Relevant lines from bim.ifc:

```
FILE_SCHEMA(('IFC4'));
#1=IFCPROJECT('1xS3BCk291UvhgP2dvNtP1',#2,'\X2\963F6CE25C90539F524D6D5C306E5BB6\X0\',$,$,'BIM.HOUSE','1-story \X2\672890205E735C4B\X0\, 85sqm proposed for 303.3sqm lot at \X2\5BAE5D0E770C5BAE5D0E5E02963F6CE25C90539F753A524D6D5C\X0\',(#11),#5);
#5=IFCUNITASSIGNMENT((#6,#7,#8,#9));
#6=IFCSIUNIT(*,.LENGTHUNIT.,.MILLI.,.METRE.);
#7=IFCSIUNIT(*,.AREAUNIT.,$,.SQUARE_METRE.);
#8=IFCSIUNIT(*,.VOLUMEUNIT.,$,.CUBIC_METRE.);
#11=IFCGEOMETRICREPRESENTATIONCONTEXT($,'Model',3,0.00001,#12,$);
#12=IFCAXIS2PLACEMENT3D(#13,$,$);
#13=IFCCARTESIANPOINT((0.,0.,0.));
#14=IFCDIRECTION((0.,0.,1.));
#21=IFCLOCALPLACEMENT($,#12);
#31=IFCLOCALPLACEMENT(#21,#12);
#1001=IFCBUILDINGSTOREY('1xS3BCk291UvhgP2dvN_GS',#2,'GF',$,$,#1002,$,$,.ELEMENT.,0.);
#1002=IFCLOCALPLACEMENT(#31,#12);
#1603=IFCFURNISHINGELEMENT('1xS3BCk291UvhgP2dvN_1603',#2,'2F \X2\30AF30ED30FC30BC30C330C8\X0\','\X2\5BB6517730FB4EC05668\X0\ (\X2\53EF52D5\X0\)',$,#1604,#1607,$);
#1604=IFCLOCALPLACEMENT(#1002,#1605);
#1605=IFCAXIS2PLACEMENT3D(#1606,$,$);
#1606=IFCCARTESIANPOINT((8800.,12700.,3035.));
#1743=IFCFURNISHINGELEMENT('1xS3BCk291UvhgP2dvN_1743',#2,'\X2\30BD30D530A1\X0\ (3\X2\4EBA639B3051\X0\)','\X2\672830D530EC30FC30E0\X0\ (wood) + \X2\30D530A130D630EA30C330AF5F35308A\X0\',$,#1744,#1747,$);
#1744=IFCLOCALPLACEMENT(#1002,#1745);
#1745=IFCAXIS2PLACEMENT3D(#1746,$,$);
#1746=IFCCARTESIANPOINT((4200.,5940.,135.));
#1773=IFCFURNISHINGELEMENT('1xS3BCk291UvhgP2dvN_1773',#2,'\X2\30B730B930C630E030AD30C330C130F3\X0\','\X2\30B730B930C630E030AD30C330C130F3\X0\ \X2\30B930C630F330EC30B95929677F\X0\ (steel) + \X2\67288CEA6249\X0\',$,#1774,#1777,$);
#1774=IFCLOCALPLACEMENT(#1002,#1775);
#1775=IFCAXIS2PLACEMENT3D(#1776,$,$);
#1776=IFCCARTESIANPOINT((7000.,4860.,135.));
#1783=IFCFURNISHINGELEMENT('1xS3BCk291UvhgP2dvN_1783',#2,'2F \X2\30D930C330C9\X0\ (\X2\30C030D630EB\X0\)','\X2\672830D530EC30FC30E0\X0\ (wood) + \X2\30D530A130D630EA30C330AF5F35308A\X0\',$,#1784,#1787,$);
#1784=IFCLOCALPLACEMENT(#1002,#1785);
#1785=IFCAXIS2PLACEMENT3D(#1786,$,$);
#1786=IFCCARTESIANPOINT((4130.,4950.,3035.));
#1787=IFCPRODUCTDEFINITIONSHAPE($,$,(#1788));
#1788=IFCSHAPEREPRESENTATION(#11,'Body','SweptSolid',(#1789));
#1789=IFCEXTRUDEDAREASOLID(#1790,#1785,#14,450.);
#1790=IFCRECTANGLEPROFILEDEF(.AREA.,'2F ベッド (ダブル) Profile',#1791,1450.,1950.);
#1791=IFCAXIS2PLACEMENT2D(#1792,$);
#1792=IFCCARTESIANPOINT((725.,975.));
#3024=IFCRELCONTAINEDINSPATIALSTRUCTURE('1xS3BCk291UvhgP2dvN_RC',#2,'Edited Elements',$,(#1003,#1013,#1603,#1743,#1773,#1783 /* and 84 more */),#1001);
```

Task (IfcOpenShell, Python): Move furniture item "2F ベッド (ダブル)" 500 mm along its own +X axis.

```python
import ifcopenshell
import ifcopenshell.api.geometry
import ifcopenshell.util.placement

model = ifcopenshell.open("bim.ifc")

item = model.by_guid("1xS3BCk291UvhgP2dvN_1783")
matrix = ifcopenshell.util.placement.get_local_placement(item.ObjectPlacement)
matrix[:3, 3] += matrix[:3, 0] * 500.0
ifcopenshell.api.geometry.edit_object_placement(model, product=item, matrix=matrix, is_si=False)

print(ifcopenshell.util.placement.get_local_placement(item.ObjectPlacement).round(3) + 0.0)

model.write("bim_updated.ifc")
```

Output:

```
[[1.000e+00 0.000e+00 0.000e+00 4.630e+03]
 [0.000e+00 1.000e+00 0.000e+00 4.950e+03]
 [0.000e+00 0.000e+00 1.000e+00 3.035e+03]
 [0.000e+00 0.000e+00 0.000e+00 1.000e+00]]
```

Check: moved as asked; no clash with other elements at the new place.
